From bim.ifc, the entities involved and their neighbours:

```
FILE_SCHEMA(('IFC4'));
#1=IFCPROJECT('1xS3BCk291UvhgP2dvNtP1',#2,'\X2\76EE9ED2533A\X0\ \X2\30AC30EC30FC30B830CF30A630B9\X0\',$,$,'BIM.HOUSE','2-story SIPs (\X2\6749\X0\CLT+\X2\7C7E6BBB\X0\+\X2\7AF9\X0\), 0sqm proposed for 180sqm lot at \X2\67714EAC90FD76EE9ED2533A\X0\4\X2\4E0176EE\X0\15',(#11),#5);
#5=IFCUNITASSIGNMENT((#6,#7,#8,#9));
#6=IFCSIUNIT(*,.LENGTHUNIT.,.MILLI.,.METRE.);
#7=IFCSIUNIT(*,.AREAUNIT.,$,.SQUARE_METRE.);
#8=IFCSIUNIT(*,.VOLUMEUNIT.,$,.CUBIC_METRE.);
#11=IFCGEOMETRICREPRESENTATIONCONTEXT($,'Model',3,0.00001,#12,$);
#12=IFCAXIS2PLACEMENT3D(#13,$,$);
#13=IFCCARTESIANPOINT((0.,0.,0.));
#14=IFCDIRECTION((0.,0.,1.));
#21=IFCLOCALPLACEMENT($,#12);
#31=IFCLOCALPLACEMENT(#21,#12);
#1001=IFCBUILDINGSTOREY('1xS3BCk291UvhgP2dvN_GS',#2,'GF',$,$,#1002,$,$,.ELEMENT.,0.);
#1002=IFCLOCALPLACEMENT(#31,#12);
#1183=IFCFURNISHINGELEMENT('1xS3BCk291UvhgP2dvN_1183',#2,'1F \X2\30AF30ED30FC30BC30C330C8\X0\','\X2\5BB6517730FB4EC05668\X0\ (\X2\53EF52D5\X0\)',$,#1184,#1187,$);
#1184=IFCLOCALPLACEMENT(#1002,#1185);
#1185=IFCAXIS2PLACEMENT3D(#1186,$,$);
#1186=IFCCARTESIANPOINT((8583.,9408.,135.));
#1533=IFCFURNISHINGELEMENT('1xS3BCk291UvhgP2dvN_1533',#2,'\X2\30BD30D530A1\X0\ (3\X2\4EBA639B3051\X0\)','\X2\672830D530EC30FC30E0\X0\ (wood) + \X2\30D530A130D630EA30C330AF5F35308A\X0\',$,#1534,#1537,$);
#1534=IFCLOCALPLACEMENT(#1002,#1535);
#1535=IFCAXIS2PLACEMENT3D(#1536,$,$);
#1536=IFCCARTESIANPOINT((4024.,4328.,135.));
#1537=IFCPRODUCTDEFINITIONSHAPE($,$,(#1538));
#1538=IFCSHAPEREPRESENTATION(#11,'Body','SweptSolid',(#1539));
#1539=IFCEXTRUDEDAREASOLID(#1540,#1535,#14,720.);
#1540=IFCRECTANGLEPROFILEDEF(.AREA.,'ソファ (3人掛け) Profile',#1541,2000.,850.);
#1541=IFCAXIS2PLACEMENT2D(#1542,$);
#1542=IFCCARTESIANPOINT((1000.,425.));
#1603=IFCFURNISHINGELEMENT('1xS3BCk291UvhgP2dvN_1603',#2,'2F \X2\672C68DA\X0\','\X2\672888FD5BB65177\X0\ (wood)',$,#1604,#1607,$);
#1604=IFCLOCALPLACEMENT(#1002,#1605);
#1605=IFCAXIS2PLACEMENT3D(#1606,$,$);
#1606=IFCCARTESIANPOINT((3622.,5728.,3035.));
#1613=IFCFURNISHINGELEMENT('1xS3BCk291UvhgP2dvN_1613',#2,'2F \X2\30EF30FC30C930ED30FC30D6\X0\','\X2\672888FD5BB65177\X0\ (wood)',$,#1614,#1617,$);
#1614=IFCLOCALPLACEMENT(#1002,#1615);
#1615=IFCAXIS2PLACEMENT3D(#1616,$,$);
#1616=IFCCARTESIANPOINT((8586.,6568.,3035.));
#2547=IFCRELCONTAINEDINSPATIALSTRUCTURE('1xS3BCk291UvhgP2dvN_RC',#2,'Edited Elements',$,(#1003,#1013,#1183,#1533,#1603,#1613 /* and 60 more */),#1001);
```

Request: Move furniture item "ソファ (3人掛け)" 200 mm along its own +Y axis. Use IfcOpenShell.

```python
import ifcopenshell
import ifcopenshell.api.geometry
import ifcopenshell.util.placement
import ifcopenshell.util.unit

model = ifcopenshell.open("bim.ifc")
unit_scale = ifcopenshell.util.unit.calculate_unit_scale(model)

item = model.by_guid("1xS3BCk291UvhgP2dvN_1533")
matrix = ifcopenshell.util.placement.get_local_placement(item.ObjectPlacement)
matrix[:3, 3] += matrix[:3, 1] * 0.2 / unit_scale
ifcopenshell.api.geometry.edit_object_placement(model, product=item, matrix=matrix, is_si=False)

print(ifcopenshell.util.placement.get_local_placement(item.ObjectPlacement).round(3) + 0.0)

model.write("bim_updated.ifc")
```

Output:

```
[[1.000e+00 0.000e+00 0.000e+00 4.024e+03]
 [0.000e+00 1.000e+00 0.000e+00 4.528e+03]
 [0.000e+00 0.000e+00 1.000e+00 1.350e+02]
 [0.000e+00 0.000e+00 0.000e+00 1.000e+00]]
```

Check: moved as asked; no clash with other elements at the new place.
